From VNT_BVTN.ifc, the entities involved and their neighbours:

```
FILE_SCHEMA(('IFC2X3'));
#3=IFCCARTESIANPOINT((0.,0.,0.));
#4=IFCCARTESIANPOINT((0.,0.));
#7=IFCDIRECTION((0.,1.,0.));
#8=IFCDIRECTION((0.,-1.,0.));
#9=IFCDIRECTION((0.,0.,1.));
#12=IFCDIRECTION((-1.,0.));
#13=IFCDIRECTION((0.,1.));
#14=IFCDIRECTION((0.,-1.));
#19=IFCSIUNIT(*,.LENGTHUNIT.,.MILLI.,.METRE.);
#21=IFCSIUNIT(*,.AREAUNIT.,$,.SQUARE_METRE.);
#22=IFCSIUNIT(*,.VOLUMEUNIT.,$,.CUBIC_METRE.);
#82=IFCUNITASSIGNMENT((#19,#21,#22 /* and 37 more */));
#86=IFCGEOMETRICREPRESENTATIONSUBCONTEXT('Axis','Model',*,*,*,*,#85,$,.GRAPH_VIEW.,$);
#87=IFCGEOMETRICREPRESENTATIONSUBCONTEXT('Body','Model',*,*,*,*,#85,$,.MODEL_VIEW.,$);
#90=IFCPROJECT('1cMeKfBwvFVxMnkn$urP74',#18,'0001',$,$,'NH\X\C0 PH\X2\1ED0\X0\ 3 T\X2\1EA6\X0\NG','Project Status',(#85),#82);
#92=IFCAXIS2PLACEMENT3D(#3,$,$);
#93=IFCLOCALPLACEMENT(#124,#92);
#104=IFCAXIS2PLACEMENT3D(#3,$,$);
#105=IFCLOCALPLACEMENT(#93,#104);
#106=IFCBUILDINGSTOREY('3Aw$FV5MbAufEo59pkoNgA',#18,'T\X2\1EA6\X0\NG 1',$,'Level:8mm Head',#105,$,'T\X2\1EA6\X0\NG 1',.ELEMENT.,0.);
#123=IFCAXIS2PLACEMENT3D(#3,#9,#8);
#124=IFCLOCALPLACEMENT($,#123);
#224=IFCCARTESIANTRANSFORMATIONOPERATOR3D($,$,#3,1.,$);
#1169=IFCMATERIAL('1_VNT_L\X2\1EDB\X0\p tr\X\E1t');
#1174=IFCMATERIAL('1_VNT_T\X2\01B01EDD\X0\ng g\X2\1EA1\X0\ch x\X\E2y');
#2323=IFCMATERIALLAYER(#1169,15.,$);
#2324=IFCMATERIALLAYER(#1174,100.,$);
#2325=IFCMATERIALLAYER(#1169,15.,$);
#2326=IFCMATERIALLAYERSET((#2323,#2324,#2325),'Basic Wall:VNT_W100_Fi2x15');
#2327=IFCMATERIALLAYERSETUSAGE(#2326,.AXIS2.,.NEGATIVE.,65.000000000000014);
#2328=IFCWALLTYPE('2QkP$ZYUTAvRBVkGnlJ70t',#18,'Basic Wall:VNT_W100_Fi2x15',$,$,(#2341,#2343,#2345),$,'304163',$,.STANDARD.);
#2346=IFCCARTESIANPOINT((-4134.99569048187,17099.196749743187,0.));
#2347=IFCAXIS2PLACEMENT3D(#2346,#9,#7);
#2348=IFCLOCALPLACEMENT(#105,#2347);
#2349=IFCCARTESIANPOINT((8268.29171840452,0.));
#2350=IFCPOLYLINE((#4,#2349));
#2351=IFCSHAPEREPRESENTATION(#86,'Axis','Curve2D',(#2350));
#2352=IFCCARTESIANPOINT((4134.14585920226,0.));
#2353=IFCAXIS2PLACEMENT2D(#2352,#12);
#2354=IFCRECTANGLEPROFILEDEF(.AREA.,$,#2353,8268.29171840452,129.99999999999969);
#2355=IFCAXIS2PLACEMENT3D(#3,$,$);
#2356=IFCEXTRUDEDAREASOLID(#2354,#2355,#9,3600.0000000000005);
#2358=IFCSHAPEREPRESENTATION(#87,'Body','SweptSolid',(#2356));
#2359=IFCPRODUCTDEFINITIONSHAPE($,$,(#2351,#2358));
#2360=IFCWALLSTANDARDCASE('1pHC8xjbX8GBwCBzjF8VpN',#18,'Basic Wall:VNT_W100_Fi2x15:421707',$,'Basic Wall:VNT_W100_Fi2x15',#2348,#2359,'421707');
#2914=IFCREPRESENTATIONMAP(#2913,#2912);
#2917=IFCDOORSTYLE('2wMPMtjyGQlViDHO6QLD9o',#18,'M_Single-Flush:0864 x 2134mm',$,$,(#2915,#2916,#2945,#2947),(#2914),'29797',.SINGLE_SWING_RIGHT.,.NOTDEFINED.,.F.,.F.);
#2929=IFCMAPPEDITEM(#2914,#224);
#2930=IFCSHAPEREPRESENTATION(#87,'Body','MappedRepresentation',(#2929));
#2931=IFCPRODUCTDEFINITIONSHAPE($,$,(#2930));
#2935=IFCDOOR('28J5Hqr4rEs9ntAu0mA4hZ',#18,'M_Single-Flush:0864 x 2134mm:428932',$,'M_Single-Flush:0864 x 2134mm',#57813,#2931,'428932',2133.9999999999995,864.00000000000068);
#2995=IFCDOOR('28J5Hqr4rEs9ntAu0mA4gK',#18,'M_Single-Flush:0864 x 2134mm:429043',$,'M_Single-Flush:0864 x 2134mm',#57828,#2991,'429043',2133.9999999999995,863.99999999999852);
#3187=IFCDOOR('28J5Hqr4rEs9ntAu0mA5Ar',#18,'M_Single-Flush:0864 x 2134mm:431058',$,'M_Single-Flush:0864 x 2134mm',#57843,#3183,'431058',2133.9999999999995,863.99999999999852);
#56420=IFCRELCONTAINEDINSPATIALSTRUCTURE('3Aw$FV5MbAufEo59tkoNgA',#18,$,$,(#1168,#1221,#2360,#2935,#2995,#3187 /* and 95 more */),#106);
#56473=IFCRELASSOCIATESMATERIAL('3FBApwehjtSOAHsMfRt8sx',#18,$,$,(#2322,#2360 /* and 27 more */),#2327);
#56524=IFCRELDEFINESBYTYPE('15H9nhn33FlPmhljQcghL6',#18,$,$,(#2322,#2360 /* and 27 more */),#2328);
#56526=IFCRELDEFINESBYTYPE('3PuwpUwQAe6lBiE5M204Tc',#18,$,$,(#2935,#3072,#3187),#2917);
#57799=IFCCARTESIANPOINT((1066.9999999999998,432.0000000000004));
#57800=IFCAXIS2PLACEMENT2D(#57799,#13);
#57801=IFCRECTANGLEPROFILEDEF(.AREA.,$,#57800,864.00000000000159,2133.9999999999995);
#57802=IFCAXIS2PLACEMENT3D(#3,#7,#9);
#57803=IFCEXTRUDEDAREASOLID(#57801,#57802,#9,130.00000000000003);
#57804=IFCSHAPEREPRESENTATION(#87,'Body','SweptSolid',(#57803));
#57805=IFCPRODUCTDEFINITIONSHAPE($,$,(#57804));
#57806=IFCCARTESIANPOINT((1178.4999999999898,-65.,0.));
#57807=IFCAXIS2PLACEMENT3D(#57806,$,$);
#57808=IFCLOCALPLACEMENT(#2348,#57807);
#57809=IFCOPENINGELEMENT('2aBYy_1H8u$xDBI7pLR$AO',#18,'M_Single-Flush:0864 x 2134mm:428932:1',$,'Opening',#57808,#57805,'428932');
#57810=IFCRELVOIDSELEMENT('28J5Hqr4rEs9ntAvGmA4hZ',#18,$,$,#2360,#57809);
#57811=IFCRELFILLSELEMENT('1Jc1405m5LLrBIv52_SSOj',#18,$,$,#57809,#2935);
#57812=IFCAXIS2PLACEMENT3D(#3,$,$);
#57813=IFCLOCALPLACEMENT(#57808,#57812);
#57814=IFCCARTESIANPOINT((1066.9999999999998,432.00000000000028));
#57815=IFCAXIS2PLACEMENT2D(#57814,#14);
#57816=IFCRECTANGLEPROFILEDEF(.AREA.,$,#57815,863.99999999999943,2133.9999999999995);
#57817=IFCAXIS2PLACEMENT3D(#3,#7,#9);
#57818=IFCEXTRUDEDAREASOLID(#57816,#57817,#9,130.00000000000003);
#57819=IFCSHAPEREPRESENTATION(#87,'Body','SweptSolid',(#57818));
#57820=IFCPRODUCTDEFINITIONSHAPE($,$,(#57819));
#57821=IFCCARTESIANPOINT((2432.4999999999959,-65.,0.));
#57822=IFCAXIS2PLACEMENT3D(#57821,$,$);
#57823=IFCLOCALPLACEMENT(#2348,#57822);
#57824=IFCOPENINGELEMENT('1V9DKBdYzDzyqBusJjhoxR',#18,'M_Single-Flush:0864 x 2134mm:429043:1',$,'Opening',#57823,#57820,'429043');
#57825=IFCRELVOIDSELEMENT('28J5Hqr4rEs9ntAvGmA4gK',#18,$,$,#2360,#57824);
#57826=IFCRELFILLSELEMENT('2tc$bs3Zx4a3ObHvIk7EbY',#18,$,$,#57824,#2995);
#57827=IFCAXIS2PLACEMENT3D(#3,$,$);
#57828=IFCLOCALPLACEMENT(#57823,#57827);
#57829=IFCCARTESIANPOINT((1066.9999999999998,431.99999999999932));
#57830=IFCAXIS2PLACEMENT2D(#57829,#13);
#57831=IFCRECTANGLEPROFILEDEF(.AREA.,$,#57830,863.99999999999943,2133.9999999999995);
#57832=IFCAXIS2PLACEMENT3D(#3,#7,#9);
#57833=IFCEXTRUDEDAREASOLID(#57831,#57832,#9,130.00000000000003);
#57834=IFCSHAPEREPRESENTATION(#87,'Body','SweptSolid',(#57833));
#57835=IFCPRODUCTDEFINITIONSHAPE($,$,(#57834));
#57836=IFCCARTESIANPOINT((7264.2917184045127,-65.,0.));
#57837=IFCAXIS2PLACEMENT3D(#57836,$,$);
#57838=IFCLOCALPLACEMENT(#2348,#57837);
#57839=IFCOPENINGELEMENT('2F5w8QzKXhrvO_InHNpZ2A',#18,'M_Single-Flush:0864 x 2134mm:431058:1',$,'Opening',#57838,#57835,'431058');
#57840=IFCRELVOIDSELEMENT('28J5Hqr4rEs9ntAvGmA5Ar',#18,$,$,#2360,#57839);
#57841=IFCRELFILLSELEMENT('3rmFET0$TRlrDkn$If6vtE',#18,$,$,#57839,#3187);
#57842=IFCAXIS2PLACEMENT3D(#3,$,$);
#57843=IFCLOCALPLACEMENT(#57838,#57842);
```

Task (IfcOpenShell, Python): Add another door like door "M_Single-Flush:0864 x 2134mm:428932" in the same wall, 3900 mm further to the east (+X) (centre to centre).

```python
import ifcopenshell
import ifcopenshell.api.feature
import ifcopenshell.api.geometry
import ifcopenshell.api.root
import ifcopenshell.geom
import ifcopenshell.util.element
import ifcopenshell.util.placement
import ifcopenshell.util.shape
import ifcopenshell.util.unit

model = ifcopenshell.open("VNT_BVTN.ifc")
unit_scale = ifcopenshell.util.unit.calculate_unit_scale(model)
settings = ifcopenshell.geom.settings()


def volume(element):
    """Net volume in cubic metres, openings subtracted."""
    shape = ifcopenshell.geom.create_shape(settings, element)
    return ifcopenshell.util.shape.get_volume(shape.geometry)


def reuse_history(source, copy):
    """copy_class also copies each property set's owner history, people and application; keep the originals."""
    for rel in copy.IsDefinedBy:
        if rel.is_a("IfcRelDefinesByProperties") and (history := rel.RelatingPropertyDefinition.OwnerHistory):
            rel.RelatingPropertyDefinition.OwnerHistory = source.OwnerHistory
            ifcopenshell.util.element.remove_deep2(model, history)


door = model.by_guid("28J5Hqr4rEs9ntAu0mA4hZ")
opening = door.FillsVoids[0].RelatingOpeningElement
wall = opening.VoidsElements[0].RelatingBuildingElement
before = volume(wall)
shift = ifcopenshell.util.placement.get_local_placement(wall.ObjectPlacement)[:3, 0] * 3.9 / unit_scale

# copy_class copies the void relationship, type, container and properties, but no geometry.
new_opening = ifcopenshell.api.root.copy_class(model, product=opening)
new_opening.Representation = ifcopenshell.util.element.copy_deep(
    model, opening.Representation, exclude=["IfcGeometricRepresentationContext", "IfcRepresentationMap"]
)
new_opening.Name = "M_Single-Flush:0864 x 2134mm"
new_opening.Tag = None
new_door = ifcopenshell.api.root.copy_class(model, product=door)
new_door.Representation = ifcopenshell.util.element.copy_deep(
    model, door.Representation, exclude=["IfcGeometricRepresentationContext", "IfcRepresentationMap"]
)
new_door.Name = "M_Single-Flush:0864 x 2134mm"
new_door.Tag = None
reuse_history(door, new_door)
fills = ifcopenshell.api.feature.add_filling(model, opening=new_opening, element=new_door)
fills.OwnerHistory = new_door.OwnerHistory  # required in IFC2X3

for old, new in ((opening, new_opening), (door, new_door)):
    matrix = ifcopenshell.util.placement.get_local_placement(old.ObjectPlacement)
    matrix[:3, 3] += shift
    ifcopenshell.api.geometry.edit_object_placement(model, product=new, matrix=matrix, is_si=False)

after = volume(wall)

print(f"wall volume {before:.3f} -> {after:.3f} m3")

model.write("VNT_BVTN_v2.ifc")
```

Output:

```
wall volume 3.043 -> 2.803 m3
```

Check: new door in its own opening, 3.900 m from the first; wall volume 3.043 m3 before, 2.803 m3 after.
